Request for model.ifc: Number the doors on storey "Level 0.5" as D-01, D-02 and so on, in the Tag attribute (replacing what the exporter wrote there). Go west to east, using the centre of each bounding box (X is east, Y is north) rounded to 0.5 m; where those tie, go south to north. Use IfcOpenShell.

First a look at what the model holds.

```python
import ifcopenshell
import ifcopenshell.util.element
import ifcopenshell.util.placement

model = ifcopenshell.open("model.ifc")
print(model.schema)
storey = next(s for s in model.by_type("IfcBuildingStorey") if s.Name == "Level 0.5")
doors = [e for e in ifcopenshell.util.element.get_decomposition(storey) if e.is_a("IfcDoor")]
for e in sorted(doors, key=lambda e: e.id()):
    origin = ifcopenshell.util.placement.get_local_placement(e.ObjectPlacement)[:3, 3]
    print(e.id(), e.Tag, e.Name, origin.round(2) + 0.0, sep=" | ")
```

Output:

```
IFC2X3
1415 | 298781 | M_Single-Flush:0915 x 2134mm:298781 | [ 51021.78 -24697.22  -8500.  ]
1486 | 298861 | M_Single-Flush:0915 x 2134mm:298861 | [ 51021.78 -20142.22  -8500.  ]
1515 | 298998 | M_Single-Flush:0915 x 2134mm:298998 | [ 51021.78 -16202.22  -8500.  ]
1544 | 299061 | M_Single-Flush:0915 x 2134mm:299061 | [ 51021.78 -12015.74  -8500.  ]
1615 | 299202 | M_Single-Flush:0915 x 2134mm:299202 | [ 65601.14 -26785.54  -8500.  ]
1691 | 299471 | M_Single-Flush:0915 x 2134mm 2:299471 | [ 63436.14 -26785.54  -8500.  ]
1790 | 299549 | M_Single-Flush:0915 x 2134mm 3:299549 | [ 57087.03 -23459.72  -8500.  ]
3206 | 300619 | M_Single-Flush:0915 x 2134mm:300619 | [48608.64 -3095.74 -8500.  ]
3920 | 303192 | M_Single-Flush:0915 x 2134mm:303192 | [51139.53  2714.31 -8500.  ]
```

```python
import ifcopenshell
import ifcopenshell.geom
import ifcopenshell.util.element
import ifcopenshell.util.shape

model = ifcopenshell.open("model.ifc")
settings = ifcopenshell.geom.settings()
settings.set("use-world-coords", True)


def centre(element):
    shape = ifcopenshell.geom.create_shape(settings, element)
    return ifcopenshell.util.shape.get_bbox_centroid(shape.geometry)


storey = next(s for s in model.by_type("IfcBuildingStorey") if s.Name == "Level 0.5")
doors = [e for e in ifcopenshell.util.element.get_decomposition(storey) if e.is_a("IfcDoor")]

# Insertion points can sit at a corner or the storey origin, so sort by the geometry (in metres).
centres = {e: centre(e) for e in doors}
doors.sort(key=lambda e: (round(centres[e][0] / 0.5), centres[e][1]))

for i, e in enumerate(doors, start=1):
    number = f"D-{i:02d}"
    e.Tag = number
    print(e.id(), number)

model.write("model-out.ifc")
```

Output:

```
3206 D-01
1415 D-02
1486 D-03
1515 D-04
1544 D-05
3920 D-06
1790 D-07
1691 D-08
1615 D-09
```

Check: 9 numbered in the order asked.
